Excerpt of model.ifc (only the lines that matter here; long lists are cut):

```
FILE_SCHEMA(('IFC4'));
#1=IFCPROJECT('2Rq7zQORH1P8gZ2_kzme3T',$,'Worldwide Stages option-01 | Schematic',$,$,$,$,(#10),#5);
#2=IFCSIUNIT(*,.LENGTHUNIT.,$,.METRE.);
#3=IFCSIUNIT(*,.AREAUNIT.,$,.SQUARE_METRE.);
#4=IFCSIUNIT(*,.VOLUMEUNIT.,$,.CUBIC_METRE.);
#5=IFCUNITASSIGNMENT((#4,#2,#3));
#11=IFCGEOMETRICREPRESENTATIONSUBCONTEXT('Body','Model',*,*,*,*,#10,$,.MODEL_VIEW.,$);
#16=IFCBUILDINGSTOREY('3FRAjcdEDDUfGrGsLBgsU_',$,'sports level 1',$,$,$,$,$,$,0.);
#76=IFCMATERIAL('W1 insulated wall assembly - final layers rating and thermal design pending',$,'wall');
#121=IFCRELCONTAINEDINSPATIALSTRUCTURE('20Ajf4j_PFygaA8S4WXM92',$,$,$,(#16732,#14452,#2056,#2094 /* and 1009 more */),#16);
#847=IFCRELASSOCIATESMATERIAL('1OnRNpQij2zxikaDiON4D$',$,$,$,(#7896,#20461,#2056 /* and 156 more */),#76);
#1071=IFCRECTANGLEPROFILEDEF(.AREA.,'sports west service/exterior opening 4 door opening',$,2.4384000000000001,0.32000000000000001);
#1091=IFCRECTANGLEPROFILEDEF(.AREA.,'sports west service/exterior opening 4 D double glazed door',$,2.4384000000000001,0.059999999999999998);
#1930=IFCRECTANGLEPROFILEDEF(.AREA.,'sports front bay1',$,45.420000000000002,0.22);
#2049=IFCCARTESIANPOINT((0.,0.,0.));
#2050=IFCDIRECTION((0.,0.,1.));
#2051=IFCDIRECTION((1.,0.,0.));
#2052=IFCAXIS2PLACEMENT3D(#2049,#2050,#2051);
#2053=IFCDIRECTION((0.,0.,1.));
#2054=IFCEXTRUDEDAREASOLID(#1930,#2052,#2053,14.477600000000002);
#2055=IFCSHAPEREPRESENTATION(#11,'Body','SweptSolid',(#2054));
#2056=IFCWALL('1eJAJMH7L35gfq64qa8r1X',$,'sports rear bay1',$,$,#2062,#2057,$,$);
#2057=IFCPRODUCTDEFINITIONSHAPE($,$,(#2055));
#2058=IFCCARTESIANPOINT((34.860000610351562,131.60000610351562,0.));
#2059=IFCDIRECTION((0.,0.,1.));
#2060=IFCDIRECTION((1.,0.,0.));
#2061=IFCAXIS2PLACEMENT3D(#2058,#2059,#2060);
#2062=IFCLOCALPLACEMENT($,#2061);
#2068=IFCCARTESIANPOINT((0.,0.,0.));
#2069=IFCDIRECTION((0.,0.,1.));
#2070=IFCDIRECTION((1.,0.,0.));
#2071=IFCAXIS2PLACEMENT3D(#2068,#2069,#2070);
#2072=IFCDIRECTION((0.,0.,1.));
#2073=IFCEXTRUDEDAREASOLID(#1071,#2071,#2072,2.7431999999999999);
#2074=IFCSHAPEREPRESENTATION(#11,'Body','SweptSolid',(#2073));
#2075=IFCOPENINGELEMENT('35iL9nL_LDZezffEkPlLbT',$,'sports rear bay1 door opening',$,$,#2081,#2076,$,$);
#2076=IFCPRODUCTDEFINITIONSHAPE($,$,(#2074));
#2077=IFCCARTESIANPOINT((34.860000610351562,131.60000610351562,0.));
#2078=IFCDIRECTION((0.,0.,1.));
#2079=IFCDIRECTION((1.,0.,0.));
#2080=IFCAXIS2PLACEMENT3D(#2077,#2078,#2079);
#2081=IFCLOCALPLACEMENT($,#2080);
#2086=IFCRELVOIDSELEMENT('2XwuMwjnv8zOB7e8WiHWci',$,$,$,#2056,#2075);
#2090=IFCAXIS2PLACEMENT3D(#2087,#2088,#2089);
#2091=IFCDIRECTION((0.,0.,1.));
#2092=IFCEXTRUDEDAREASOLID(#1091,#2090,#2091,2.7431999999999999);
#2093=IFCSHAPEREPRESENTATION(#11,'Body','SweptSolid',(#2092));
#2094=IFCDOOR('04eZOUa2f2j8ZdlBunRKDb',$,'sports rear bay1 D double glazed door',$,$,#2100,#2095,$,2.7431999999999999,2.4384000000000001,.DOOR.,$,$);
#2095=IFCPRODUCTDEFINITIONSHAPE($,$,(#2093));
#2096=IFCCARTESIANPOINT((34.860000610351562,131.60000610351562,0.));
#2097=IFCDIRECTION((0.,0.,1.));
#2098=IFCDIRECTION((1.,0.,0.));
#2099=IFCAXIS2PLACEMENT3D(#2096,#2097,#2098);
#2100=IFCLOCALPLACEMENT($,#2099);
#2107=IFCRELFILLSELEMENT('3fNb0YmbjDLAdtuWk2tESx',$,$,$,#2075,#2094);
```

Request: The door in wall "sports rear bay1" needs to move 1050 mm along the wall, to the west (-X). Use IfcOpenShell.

```python
import ifcopenshell
import ifcopenshell.api.geometry
import ifcopenshell.util.placement
import ifcopenshell.util.unit

model = ifcopenshell.open("model.ifc")
unit_scale = ifcopenshell.util.unit.calculate_unit_scale(model)

door = model.by_id(2094)
opening = door.FillsVoids[0].RelatingOpeningElement
wall = opening.VoidsElements[0].RelatingBuildingElement

wall_matrix = ifcopenshell.util.placement.get_local_placement(wall.ObjectPlacement)
shift = wall_matrix[:3, 0] * -1.05 / unit_scale
before = ifcopenshell.util.placement.get_local_placement(door.ObjectPlacement)[:3, 3].copy()

# The door is not placed relative to its opening, so move both.
for product in (opening, door):
    matrix = ifcopenshell.util.placement.get_local_placement(product.ObjectPlacement)
    matrix[:3, 3] += shift
    ifcopenshell.api.geometry.edit_object_placement(model, product=product, matrix=matrix, is_si=False)

after = ifcopenshell.util.placement.get_local_placement(door.ObjectPlacement)[:3, 3]
print("door moved by", (after - before).round(3) + 0.0)

model.write("model-out.ifc")
```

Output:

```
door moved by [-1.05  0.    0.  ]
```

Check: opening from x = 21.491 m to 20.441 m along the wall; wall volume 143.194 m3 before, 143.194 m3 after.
